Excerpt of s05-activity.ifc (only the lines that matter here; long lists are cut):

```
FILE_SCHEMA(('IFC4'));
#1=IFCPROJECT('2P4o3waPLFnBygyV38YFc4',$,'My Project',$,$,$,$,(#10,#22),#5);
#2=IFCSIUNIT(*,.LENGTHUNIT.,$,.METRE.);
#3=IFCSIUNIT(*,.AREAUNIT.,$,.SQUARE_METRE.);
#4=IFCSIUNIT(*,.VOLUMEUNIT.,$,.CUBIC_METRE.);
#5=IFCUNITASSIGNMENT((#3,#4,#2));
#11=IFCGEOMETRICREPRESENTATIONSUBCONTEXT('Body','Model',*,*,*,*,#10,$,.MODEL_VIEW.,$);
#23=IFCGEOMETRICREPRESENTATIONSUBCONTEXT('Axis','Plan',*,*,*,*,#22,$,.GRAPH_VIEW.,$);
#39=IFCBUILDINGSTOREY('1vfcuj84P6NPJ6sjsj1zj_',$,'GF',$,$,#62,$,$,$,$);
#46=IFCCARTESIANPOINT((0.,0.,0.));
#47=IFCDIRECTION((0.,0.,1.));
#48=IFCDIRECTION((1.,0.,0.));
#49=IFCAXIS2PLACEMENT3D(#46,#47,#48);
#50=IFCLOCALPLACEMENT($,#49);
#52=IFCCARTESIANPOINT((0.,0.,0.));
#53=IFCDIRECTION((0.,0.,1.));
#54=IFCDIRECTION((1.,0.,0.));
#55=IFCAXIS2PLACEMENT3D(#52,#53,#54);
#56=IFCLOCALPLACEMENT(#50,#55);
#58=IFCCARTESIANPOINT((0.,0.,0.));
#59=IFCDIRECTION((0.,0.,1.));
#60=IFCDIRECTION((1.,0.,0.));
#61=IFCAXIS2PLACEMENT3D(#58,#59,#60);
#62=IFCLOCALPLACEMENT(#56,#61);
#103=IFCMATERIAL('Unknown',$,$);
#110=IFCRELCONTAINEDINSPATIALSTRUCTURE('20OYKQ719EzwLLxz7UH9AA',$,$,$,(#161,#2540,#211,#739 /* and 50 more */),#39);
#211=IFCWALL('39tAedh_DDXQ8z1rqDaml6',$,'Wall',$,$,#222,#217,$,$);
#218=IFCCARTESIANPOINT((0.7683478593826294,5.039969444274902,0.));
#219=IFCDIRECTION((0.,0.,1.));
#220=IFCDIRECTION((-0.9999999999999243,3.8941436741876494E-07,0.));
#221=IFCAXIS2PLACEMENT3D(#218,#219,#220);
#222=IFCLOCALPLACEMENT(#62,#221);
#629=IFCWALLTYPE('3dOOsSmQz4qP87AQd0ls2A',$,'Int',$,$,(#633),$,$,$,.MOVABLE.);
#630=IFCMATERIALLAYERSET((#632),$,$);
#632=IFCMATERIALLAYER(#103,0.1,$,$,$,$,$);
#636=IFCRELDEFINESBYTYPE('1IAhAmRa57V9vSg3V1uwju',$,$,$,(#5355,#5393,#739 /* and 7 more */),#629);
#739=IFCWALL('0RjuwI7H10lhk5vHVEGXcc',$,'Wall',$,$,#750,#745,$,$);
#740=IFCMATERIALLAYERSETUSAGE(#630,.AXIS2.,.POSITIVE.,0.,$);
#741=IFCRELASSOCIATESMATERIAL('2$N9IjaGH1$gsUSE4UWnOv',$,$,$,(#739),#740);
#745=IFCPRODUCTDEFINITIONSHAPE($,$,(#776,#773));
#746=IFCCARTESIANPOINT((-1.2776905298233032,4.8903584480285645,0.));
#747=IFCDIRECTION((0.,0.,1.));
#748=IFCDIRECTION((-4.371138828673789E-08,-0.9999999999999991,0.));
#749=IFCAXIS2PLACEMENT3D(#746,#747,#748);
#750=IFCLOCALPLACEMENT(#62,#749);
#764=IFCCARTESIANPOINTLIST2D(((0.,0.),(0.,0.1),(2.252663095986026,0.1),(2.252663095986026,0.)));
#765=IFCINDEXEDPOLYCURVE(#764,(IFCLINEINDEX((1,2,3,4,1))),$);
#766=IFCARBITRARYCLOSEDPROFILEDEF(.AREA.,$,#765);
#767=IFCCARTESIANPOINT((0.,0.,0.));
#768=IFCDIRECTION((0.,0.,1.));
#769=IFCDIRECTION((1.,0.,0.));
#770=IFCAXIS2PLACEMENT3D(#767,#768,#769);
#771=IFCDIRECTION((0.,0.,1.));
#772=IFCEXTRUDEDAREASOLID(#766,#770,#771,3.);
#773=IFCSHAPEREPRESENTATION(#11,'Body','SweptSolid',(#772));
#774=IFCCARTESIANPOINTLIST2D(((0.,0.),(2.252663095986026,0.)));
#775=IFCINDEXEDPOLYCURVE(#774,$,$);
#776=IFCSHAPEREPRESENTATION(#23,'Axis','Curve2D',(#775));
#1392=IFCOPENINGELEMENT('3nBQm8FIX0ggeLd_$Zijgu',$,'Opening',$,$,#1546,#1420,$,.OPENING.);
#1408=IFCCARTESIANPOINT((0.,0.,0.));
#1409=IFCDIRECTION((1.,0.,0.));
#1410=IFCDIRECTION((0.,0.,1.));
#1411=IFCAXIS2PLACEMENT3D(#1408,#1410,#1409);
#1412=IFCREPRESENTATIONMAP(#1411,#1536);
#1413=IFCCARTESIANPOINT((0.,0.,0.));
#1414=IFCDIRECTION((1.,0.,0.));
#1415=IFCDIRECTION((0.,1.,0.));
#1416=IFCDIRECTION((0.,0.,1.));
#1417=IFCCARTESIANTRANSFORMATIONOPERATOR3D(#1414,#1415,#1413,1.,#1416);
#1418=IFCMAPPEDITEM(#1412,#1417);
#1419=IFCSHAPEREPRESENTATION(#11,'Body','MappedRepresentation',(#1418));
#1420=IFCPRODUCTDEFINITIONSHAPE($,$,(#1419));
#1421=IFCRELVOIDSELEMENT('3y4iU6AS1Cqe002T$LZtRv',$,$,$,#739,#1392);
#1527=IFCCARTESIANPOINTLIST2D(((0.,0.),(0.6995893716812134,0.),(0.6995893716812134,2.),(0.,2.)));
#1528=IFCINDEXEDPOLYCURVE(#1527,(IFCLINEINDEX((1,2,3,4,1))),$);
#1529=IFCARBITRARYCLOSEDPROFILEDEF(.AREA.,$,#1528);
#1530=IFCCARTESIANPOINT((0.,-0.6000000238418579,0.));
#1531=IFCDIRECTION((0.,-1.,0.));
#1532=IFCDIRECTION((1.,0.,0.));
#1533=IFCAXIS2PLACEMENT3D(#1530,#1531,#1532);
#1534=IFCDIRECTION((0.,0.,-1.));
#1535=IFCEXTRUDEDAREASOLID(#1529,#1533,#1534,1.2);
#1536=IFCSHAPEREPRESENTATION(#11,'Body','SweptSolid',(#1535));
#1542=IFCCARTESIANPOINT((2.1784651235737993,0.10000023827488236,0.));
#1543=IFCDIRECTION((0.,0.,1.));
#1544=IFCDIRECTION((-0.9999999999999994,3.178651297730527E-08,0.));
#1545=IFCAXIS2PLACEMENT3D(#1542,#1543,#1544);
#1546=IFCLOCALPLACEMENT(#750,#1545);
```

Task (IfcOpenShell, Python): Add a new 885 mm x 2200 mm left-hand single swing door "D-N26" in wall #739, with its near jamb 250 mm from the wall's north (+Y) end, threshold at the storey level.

```python
import numpy as np
import ifcopenshell
import ifcopenshell.api.feature
import ifcopenshell.api.geometry
import ifcopenshell.api.root
import ifcopenshell.api.spatial
import ifcopenshell.geom
import ifcopenshell.util.element
import ifcopenshell.util.placement
import ifcopenshell.util.representation
import ifcopenshell.util.shape
import ifcopenshell.util.unit

model = ifcopenshell.open("s05-activity.ifc")
unit_scale = ifcopenshell.util.unit.calculate_unit_scale(model)
settings = ifcopenshell.geom.settings()


def volume(element):
    """Net volume in cubic metres, openings subtracted."""
    shape = ifcopenshell.geom.create_shape(settings, element)
    return ifcopenshell.util.shape.get_volume(shape.geometry)


wall = model.by_guid("0RjuwI7H10lhk5vHVEGXcc")
storey = ifcopenshell.util.element.get_container(wall, ifc_class="IfcBuildingStorey")
context = ifcopenshell.util.representation.get_context(model, "Model", "Body", "MODEL_VIEW")
before = volume(wall)

width, height, from_end, sill = 0.885, 2.2, 0.25, 0.0  # metres

# The wall runs along its own X axis, and the end named is its -X end.
wall_shape = ifcopenshell.geom.create_shape(settings, wall)
x, y, z = ifcopenshell.util.shape.get_vertices(wall_shape.geometry).T
start = x.min() + from_end
face, thickness = float(y.min()), float(y.max() - y.min())
wall_matrix = ifcopenshell.util.placement.get_local_placement(wall.ObjectPlacement)
level = ifcopenshell.util.placement.get_local_placement(storey.ObjectPlacement)[2, 3]


def in_wall(x, y):
    """Placement at x, y metres in the wall's axes, at sill height."""
    matrix = wall_matrix.copy()
    matrix[:, 3] = wall_matrix @ np.array([x / unit_scale, y / unit_scale, 0.0, 1.0])
    matrix[2, 3] = level + sill / unit_scale
    return matrix


# Opening: a box that overshoots both wall faces by 50 mm.
opening = ifcopenshell.api.root.create_entity(model, ifc_class="IfcOpeningElement", predefined_type="OPENING")
box = ifcopenshell.api.geometry.add_wall_representation(
    model, context=context, length=width, height=height, thickness=thickness + 0.1
)
ifcopenshell.api.geometry.assign_representation(model, product=opening, representation=box)
ifcopenshell.api.geometry.edit_object_placement(model, product=opening, matrix=in_wall(start, face - 0.05), is_si=False)
ifcopenshell.api.feature.add_feature(model, feature=opening, element=wall)

door = ifcopenshell.api.root.create_entity(model, ifc_class="IfcDoor", name="D-N26", predefined_type="DOOR")
door.OverallWidth, door.OverallHeight = width / unit_scale, height / unit_scale
door.OperationType = "SINGLE_SWING_LEFT"
body = ifcopenshell.api.geometry.add_door_representation(
    model,
    context=context,
    overall_width=door.OverallWidth,
    overall_height=door.OverallHeight,
    operation_type="SINGLE_SWING_LEFT",
    lining_properties={"LiningDepth": thickness / unit_scale, "ThresholdDepth": thickness / unit_scale},
)
ifcopenshell.api.geometry.assign_representation(model, product=door, representation=body)
ifcopenshell.api.spatial.assign_container(model, products=[door], relating_structure=storey)
ifcopenshell.api.feature.add_filling(model, opening=opening, element=door)

# The lining spans the wall, so the door starts at the wall face.
ifcopenshell.api.geometry.edit_object_placement(model, product=door, matrix=in_wall(start, face), is_si=False)

after = volume(wall)

print(f"wall volume {before:.3f} -> {after:.3f} m3")

model.write("s05-activity_updated.ifc")
```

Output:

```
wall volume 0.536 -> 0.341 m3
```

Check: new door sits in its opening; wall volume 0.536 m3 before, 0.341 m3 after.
